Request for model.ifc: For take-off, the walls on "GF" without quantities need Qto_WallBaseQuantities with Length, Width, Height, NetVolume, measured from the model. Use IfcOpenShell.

First a look at what the model holds.

```python
import ifcopenshell
import ifcopenshell.util.element
import ifcopenshell.util.unit

model = ifcopenshell.open("model.ifc")
print(model.schema)
for unit_type in ("LENGTHUNIT", "AREAUNIT", "VOLUMEUNIT"):
    print(unit_type, ifcopenshell.util.unit.calculate_unit_scale(model, unit_type))
storey = next(s for s in model.by_type("IfcBuildingStorey") if s.Name == "GF")
walls = [e for e in ifcopenshell.util.element.get_decomposition(storey) if e.is_a("IfcWall")]
for e in sorted(walls, key=lambda e: e.id()):
    print(e.id(), e.is_a(), e.Name, list(ifcopenshell.util.element.get_psets(e, qtos_only=True)), sep=" | ")
```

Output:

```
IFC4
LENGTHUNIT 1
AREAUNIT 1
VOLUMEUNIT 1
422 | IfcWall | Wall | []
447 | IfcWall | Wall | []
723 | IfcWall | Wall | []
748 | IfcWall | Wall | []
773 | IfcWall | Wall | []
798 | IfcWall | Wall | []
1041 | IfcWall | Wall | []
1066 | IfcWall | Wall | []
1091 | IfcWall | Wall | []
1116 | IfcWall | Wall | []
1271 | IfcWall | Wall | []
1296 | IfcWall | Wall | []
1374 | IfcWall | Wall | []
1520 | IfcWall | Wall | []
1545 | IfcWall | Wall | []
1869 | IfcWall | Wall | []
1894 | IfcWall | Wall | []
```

```python
import ifcopenshell
import ifcopenshell.api.pset
import ifcopenshell.geom
import ifcopenshell.util.element
import ifcopenshell.util.shape
import ifcopenshell.util.unit

model = ifcopenshell.open("model.ifc")
unit_scale = ifcopenshell.util.unit.calculate_unit_scale(model)
volume_scale = ifcopenshell.util.unit.calculate_unit_scale(model, "VOLUMEUNIT")
settings = ifcopenshell.geom.settings()

storey = next(s for s in model.by_type("IfcBuildingStorey") if s.Name == "GF")
walls = [e for e in ifcopenshell.util.element.get_decomposition(storey) if e.is_a("IfcWall")]

for e in sorted(walls, key=lambda e: e.id()):
    if ifcopenshell.util.element.get_psets(e, qtos_only=True, should_inherit=False):
        continue
    # Geometry comes back in metres, in the element's own axes.
    shape = ifcopenshell.geom.create_shape(settings, e)
    values = {
        "Length": ifcopenshell.util.shape.get_x(shape.geometry) / unit_scale,
        "Width": ifcopenshell.util.shape.get_y(shape.geometry) / unit_scale,
        "Height": ifcopenshell.util.shape.get_z(shape.geometry) / unit_scale,
        "NetVolume": ifcopenshell.util.shape.get_volume(shape.geometry) / volume_scale,
    }
    qto = ifcopenshell.api.pset.add_qto(model, product=e, name="Qto_WallBaseQuantities")
    ifcopenshell.api.pset.edit_qto(model, qto=qto, properties=values)
    print(e.id(), {k: round(v, 3) for k, v in values.items()})

model.write("model_updated.ifc")
```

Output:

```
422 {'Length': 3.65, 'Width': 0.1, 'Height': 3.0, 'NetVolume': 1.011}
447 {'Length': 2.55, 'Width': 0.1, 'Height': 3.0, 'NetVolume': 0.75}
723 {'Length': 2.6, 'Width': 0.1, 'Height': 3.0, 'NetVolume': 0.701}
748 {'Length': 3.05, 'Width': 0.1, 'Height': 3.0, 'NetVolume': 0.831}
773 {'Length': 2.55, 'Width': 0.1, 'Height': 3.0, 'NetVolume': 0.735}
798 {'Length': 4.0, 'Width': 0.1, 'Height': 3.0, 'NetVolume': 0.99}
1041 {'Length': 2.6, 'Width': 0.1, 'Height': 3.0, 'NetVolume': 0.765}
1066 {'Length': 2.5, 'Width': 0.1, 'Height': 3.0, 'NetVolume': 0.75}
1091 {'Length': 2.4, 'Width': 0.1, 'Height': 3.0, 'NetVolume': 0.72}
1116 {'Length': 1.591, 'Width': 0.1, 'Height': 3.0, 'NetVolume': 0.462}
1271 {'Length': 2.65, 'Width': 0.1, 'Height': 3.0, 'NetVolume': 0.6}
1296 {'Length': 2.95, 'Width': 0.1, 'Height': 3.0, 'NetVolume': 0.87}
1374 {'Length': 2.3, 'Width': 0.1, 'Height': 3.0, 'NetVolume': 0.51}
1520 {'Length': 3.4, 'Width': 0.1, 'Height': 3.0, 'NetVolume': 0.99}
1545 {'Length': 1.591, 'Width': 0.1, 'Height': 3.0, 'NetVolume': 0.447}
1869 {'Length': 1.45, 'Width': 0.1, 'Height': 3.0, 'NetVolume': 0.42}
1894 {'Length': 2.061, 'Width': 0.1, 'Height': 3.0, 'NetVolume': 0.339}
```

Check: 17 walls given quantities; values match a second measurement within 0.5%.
